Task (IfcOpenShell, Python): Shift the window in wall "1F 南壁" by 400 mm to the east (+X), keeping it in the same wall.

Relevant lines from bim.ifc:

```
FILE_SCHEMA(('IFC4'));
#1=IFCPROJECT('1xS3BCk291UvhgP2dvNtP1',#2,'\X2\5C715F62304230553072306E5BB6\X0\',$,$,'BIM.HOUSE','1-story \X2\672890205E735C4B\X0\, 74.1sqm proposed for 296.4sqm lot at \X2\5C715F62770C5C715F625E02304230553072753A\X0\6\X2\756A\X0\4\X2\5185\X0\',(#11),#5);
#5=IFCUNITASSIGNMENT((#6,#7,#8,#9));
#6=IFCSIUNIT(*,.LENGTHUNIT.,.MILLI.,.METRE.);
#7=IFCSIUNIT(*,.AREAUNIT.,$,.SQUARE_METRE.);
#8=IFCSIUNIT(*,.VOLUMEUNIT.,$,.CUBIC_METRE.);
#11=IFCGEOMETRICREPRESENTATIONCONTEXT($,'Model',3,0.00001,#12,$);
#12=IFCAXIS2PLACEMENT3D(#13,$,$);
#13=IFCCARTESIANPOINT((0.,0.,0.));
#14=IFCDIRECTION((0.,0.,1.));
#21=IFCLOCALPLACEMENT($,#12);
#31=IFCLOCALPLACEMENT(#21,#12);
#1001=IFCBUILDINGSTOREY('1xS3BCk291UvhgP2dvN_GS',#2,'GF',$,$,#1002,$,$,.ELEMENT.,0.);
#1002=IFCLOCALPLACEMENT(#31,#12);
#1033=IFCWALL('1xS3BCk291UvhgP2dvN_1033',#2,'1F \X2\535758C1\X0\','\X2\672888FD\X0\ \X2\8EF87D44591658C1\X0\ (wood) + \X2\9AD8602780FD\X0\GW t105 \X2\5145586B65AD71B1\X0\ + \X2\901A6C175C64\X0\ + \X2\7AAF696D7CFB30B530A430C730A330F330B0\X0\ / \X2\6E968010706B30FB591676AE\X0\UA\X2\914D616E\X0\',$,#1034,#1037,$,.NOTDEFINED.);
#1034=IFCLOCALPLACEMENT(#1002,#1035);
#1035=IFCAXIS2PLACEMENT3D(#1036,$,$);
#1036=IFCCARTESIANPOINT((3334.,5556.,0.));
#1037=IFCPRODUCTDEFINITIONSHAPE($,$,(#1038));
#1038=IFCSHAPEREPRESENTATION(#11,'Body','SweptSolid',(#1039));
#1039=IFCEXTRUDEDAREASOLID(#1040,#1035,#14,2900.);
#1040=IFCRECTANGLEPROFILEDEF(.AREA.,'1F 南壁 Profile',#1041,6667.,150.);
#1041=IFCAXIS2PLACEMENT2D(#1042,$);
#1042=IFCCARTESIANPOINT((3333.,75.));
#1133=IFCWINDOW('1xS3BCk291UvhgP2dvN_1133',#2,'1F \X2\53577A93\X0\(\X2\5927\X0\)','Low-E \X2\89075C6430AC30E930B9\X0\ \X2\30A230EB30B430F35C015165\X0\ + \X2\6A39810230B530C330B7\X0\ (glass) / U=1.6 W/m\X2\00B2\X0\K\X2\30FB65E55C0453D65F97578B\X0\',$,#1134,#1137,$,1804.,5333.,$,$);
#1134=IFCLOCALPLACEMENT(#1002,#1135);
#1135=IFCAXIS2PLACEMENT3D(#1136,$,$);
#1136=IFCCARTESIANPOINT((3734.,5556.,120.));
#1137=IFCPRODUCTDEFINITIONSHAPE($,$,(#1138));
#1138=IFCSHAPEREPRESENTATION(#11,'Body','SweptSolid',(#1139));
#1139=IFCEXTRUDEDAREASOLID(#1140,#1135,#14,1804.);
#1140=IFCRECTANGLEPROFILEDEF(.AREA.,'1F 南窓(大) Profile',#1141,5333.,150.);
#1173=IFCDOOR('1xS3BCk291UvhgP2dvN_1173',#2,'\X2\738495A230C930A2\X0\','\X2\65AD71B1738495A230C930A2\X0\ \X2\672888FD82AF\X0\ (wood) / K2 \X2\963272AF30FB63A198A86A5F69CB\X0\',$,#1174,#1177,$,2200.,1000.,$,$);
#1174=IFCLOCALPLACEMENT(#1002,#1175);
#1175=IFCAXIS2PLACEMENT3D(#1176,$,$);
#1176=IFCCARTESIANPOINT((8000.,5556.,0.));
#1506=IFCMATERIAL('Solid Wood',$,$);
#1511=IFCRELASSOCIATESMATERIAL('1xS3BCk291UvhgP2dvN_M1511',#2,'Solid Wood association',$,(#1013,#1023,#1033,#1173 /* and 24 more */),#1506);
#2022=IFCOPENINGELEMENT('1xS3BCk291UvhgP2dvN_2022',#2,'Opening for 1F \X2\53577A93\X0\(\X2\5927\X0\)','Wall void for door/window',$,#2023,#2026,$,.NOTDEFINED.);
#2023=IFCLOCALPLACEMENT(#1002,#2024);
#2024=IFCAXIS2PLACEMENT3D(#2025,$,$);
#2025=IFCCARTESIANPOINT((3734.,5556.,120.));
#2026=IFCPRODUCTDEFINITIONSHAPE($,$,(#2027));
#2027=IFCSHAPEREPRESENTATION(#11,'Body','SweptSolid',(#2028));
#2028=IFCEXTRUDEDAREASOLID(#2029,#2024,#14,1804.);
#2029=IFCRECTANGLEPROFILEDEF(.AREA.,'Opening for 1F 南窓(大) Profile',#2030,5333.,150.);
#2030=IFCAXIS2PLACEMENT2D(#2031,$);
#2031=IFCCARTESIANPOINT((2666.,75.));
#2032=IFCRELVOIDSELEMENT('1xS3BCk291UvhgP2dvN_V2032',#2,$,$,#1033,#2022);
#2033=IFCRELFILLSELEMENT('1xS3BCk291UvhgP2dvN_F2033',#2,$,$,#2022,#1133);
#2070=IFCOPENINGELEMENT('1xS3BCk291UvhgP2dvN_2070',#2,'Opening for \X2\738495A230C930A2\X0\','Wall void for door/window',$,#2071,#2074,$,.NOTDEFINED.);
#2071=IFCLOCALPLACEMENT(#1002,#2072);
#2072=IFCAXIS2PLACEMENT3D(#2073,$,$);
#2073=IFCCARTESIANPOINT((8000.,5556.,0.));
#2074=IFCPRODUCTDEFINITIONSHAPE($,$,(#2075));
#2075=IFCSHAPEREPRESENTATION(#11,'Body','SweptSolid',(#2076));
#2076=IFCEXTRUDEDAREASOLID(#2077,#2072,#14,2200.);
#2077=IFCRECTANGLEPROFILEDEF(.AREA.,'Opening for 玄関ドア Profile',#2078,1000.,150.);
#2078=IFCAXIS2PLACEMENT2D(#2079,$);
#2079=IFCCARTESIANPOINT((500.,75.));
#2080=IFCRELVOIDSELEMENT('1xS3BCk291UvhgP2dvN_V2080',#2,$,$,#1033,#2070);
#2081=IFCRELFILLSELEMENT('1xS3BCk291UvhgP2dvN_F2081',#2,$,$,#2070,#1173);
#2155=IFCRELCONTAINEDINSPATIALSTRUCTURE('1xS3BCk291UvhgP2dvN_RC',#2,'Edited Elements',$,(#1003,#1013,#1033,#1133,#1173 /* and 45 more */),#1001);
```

```python
import ifcopenshell
import ifcopenshell.api.geometry
import ifcopenshell.util.placement

model = ifcopenshell.open("bim.ifc")

window = model.by_id(1133)
opening = window.FillsVoids[0].RelatingOpeningElement
wall = opening.VoidsElements[0].RelatingBuildingElement

wall_matrix = ifcopenshell.util.placement.get_local_placement(wall.ObjectPlacement)
shift = wall_matrix[:3, 0] * 400.0
before = ifcopenshell.util.placement.get_local_placement(window.ObjectPlacement)[:3, 3].copy()

# The window is not placed relative to its opening, so move both.
for product in (opening, window):
    matrix = ifcopenshell.util.placement.get_local_placement(product.ObjectPlacement)
    matrix[:3, 3] += shift
    ifcopenshell.api.geometry.edit_object_placement(model, product=product, matrix=matrix, is_si=False)

after = ifcopenshell.util.placement.get_local_placement(window.ObjectPlacement)[:3, 3]
print("window moved by", (after - before).round(3) + 0.0)

model.write("bim_edited.ifc")
```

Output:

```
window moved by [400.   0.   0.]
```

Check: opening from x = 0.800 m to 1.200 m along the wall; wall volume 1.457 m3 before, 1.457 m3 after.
